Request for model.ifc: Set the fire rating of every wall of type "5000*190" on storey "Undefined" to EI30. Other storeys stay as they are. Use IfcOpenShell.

First a look at what the model holds.

```python
import ifcopenshell
import ifcopenshell.util.element

model = ifcopenshell.open("model.ifc")
print(model.schema)
storey = next(s for s in model.by_type("IfcBuildingStorey") if s.Name == "Undefined")
walls = [e for e in ifcopenshell.util.element.get_decomposition(storey) if e.is_a("IfcWall")]
seen = {}
for e in walls:
    element_type = ifcopenshell.util.element.get_type(e)
    key = (element_type.Name if element_type != e and element_type else None, ifcopenshell.util.element.get_pset(e, "Pset_WallCommon", "FireRating"))
    seen[key] = seen.get(key, 0) + 1
for (name, value), count in sorted(seen.items(), key=str):
    print(count, "x", name, "|", value)
```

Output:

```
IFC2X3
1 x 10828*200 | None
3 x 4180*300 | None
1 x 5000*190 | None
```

```python
import ifcopenshell
import ifcopenshell.api.pset
import ifcopenshell.util.element

model = ifcopenshell.open("model.ifc")

storey = next(s for s in model.by_type("IfcBuildingStorey") if s.Name == "Undefined")
walls = [e for e in ifcopenshell.util.element.get_decomposition(storey) if e.is_a("IfcWall")]

count = 0
for e in walls:
    element_type = ifcopenshell.util.element.get_type(e)
    if element_type in (None, e) or element_type.Name != "5000*190":
        continue
    found = ifcopenshell.util.element.get_pset(e, "Pset_WallCommon", should_inherit=False)
    if found:
        pset = model.by_id(found["id"])
        if len(ifcopenshell.util.element.get_elements_by_pset(pset)) > 1:
            pset = ifcopenshell.api.pset.unshare_pset(model, products=[e], pset=pset)[0]
    else:
        pset = ifcopenshell.api.pset.add_pset(model, product=e, name="Pset_WallCommon")
    ifcopenshell.api.pset.edit_pset(model, pset=pset, properties={"FireRating": "EI30"})
    count += 1

print(count, "walls updated")

model.write("model_edited.ifc")
```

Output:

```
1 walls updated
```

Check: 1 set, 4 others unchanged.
